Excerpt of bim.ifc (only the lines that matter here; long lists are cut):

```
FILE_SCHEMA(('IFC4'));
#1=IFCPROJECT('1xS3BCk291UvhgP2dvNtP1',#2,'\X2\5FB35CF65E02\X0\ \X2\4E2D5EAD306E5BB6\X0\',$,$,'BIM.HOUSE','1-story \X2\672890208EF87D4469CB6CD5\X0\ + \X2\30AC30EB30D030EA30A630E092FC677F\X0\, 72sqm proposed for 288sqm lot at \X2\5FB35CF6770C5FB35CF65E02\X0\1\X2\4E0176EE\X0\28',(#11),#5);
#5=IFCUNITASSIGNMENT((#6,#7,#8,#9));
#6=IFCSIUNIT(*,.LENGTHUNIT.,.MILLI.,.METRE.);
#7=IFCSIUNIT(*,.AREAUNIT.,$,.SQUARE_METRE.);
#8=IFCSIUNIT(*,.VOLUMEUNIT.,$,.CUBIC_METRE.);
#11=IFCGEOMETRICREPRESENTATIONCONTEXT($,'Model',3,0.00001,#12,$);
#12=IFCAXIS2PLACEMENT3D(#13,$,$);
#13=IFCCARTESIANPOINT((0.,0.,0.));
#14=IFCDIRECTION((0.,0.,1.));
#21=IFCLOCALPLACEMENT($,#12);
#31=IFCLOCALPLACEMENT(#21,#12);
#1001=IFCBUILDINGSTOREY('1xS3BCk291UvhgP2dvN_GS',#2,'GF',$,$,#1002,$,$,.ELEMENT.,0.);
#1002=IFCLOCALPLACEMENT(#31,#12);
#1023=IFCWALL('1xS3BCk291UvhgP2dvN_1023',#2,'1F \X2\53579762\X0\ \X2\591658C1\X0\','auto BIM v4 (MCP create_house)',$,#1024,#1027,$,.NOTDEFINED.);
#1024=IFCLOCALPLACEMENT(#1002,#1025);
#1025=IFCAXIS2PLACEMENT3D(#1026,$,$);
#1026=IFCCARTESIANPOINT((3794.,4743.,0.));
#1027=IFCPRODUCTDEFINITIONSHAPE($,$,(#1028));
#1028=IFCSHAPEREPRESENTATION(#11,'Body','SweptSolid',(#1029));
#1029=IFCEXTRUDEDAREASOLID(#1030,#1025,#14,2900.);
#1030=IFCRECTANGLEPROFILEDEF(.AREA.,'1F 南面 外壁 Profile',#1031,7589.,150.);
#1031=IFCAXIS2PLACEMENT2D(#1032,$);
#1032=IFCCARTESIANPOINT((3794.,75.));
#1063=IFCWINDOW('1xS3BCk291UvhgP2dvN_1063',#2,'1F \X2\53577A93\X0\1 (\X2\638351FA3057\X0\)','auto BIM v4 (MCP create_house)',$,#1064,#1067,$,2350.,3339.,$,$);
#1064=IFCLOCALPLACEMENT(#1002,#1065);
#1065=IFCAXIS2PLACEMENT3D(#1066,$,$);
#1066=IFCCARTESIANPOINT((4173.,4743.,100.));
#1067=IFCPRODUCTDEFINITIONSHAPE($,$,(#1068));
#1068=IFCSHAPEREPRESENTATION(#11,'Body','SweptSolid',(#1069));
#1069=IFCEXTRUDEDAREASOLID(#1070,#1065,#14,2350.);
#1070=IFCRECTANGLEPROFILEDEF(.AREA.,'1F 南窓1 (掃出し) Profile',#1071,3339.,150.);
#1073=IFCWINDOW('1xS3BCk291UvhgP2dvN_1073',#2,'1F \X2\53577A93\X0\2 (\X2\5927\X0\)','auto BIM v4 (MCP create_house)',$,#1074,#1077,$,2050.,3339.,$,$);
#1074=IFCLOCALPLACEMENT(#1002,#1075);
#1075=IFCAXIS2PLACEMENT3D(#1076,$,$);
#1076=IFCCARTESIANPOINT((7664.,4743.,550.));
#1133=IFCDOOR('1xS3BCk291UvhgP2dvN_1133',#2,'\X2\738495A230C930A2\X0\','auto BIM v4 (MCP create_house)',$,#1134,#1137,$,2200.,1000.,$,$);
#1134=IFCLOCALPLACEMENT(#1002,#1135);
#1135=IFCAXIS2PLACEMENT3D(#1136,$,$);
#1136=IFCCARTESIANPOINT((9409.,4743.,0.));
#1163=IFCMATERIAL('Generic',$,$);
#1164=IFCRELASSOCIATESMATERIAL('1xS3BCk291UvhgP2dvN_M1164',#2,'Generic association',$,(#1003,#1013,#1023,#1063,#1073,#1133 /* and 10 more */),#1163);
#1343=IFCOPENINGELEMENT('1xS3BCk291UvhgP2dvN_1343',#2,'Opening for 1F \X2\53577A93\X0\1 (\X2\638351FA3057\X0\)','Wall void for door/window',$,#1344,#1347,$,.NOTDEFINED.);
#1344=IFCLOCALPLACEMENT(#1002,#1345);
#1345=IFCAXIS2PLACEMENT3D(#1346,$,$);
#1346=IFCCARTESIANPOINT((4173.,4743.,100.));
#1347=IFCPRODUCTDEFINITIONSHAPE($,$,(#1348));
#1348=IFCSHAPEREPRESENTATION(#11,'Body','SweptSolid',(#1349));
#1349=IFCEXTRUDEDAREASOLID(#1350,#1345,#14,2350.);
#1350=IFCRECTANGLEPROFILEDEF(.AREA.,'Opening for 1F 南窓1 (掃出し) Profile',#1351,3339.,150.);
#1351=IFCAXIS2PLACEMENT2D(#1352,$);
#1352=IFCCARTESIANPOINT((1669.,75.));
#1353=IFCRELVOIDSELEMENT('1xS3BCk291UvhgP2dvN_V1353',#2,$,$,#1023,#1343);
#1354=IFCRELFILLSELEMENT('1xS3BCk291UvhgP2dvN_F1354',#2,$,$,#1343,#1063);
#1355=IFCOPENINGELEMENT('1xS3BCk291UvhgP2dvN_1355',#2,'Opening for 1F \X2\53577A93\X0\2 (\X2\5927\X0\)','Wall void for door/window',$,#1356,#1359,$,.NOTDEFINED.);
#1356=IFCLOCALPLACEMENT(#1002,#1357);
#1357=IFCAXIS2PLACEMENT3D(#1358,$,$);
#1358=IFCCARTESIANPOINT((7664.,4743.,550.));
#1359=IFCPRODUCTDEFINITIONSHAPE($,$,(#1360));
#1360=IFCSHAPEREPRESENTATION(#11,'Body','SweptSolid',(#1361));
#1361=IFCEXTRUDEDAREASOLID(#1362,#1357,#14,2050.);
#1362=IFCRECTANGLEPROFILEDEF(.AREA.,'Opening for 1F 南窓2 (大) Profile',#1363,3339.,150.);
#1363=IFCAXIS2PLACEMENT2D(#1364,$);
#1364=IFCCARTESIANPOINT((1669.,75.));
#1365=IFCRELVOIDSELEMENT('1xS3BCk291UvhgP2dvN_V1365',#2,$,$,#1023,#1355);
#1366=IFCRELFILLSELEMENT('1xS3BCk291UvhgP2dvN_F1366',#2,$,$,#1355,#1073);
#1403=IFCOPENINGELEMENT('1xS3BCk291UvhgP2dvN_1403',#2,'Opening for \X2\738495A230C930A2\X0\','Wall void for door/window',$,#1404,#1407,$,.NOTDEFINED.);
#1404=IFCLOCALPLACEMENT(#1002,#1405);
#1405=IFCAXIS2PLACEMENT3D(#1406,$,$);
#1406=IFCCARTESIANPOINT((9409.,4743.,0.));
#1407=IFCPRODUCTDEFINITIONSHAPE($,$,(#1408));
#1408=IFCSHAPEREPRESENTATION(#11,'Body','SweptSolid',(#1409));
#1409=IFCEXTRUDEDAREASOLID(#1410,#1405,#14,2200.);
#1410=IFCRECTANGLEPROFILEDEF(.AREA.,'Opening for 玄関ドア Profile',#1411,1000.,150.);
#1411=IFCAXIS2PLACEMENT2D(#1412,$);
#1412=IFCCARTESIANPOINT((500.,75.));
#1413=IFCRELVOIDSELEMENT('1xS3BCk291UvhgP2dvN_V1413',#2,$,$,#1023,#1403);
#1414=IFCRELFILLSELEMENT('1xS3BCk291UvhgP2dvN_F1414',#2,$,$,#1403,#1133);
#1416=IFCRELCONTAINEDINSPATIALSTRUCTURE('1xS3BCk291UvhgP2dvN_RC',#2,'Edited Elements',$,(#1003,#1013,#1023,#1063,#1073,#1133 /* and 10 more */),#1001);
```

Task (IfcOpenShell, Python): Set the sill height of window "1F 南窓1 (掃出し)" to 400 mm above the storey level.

```python
import numpy as np
import ifcopenshell
import ifcopenshell.api.geometry
import ifcopenshell.geom
import ifcopenshell.util.element
import ifcopenshell.util.placement
import ifcopenshell.util.shape
import ifcopenshell.util.unit

model = ifcopenshell.open("bim.ifc")
unit_scale = ifcopenshell.util.unit.calculate_unit_scale(model)

window = model.by_id(1063)
opening = window.FillsVoids[0].RelatingOpeningElement
storey = ifcopenshell.util.element.get_container(window, ifc_class="IfcBuildingStorey")
level = ifcopenshell.util.placement.get_local_placement(storey.ObjectPlacement)[2, 3]

# The opening's origin need not be at the sill, so measure its lowest point.
shape = ifcopenshell.geom.create_shape(ifcopenshell.geom.settings(), opening)
bottom = ifcopenshell.util.shape.get_shape_bottom_elevation(shape, shape.geometry) / unit_scale
dz = level + 400.0 - bottom

shift = np.array([0.0, 0.0, dz])
# The window is not placed relative to its opening, so move both.
for product in (opening, window):
    matrix = ifcopenshell.util.placement.get_local_placement(product.ObjectPlacement)
    matrix[:3, 3] += shift
    ifcopenshell.api.geometry.edit_object_placement(model, product=product, matrix=matrix, is_si=False)

print(f"moved by {dz * unit_scale:+.3f} m")

model.write("bim_updated.ifc")
```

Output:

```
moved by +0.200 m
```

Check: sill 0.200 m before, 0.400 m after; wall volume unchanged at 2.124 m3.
